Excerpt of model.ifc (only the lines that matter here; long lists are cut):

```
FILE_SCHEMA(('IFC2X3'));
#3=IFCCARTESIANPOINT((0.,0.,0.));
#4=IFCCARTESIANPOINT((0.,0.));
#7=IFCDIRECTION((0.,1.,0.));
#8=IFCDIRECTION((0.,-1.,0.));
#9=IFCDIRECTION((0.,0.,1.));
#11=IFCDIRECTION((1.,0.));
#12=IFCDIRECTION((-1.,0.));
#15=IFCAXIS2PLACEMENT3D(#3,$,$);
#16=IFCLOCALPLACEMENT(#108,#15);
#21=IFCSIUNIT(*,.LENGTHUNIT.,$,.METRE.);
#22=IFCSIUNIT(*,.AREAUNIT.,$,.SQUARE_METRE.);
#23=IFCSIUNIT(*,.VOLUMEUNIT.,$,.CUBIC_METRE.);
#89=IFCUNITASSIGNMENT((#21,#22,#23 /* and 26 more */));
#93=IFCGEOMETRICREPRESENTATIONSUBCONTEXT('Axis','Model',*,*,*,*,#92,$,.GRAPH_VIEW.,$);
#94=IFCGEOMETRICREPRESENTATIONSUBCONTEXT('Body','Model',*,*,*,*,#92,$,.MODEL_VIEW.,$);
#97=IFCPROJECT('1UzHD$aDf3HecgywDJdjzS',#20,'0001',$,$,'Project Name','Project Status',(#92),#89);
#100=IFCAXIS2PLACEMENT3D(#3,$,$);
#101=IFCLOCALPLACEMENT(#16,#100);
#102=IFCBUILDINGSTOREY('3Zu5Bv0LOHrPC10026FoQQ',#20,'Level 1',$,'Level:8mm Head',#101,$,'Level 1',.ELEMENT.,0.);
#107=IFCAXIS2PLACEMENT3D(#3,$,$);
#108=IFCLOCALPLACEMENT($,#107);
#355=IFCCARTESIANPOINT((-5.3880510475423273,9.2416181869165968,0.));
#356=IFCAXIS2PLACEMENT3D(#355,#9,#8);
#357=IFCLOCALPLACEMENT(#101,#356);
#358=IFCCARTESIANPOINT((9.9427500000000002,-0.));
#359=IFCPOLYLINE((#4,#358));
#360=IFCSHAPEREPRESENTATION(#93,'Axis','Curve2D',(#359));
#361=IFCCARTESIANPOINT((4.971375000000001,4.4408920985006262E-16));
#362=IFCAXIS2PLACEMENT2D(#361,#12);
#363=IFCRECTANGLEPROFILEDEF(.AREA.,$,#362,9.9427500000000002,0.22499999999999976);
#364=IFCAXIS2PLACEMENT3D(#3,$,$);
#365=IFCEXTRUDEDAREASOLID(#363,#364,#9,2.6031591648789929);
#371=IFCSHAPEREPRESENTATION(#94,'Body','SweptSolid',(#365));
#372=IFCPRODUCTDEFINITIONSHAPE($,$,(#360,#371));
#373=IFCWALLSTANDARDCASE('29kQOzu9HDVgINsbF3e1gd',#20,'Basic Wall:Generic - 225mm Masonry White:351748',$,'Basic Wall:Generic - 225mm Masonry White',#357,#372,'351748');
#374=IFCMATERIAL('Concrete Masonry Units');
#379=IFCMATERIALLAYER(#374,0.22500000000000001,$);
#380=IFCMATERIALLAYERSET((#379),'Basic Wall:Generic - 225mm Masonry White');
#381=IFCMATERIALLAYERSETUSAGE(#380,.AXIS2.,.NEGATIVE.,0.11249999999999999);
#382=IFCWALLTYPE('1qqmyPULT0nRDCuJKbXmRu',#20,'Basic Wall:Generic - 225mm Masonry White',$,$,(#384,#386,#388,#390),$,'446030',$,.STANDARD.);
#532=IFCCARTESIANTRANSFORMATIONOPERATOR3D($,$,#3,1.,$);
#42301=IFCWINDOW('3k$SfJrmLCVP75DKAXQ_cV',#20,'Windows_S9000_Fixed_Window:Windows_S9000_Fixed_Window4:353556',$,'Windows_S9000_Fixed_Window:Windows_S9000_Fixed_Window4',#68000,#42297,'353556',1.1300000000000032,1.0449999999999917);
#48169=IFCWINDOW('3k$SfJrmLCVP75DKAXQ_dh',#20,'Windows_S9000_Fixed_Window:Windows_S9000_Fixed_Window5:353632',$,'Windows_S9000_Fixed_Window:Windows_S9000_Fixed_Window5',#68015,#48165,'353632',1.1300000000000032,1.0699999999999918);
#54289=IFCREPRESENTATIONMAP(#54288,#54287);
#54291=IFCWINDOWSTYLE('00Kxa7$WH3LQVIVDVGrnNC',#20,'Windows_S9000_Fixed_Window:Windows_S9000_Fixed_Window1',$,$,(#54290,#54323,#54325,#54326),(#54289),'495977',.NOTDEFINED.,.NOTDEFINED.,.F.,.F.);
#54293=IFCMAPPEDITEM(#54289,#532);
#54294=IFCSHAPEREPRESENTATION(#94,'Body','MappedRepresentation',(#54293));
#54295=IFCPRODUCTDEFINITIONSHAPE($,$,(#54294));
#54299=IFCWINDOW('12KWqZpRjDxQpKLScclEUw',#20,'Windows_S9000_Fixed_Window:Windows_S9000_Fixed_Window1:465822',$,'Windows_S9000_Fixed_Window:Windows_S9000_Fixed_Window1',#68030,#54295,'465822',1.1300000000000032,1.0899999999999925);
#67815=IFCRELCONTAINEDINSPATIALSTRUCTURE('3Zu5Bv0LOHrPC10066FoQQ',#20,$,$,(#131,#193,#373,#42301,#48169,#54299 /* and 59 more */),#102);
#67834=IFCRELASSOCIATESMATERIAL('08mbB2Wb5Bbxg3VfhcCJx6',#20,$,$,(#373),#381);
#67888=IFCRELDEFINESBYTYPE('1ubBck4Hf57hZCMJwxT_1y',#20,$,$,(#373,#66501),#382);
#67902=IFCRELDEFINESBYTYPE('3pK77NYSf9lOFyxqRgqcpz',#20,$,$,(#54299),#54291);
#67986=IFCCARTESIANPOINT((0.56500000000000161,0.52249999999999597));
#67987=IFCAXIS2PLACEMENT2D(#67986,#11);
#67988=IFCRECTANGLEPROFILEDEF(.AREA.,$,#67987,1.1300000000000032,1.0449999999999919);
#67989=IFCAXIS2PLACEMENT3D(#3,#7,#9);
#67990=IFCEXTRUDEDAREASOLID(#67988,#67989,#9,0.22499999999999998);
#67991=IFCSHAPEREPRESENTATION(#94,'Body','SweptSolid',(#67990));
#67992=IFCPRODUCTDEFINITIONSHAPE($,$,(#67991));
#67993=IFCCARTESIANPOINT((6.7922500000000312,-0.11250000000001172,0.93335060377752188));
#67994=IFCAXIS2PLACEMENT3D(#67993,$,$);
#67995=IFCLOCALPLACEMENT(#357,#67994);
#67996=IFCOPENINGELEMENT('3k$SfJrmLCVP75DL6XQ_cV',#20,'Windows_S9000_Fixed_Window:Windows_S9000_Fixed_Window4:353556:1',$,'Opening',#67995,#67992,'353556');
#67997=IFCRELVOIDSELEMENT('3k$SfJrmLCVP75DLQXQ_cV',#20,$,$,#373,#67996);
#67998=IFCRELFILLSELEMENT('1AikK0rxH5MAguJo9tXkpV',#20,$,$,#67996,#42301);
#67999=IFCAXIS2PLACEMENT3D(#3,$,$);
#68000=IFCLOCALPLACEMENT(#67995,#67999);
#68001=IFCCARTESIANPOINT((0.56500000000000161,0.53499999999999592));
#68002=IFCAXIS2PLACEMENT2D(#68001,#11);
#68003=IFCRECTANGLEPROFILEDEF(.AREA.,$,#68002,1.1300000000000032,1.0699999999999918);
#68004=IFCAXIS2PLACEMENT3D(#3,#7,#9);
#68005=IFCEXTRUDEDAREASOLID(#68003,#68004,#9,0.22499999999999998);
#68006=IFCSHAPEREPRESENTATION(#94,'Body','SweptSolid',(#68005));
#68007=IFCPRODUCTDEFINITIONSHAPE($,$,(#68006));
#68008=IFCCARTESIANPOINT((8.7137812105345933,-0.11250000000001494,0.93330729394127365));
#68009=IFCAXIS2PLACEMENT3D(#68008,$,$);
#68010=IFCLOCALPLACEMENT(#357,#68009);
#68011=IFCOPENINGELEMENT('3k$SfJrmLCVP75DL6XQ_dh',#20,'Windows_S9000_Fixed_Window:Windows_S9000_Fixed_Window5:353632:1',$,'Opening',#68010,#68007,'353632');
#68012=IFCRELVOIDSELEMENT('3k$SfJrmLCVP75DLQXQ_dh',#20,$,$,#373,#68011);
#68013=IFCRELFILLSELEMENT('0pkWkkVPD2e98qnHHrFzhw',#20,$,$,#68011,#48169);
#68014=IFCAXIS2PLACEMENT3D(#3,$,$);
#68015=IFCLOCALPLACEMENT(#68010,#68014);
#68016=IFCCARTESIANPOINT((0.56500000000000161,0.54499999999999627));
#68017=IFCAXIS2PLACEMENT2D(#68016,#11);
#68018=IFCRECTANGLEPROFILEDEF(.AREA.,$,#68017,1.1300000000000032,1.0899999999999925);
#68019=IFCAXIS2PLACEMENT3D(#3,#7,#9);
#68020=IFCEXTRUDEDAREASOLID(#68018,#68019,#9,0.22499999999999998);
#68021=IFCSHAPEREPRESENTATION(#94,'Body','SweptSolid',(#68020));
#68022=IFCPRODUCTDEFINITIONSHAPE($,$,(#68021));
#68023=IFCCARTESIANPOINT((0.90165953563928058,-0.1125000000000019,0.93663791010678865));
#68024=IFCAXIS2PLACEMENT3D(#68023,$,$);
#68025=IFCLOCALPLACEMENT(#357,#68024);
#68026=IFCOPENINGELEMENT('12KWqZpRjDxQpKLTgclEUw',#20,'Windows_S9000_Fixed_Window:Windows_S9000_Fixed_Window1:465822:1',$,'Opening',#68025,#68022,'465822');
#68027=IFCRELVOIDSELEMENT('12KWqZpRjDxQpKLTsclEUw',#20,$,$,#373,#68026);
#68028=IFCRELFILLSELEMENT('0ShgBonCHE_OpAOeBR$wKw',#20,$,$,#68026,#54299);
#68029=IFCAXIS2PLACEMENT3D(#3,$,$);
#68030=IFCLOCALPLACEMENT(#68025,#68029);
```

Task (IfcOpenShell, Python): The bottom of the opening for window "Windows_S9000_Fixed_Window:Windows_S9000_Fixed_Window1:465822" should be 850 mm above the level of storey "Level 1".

```python
import numpy as np
import ifcopenshell
import ifcopenshell.api.geometry
import ifcopenshell.geom
import ifcopenshell.util.element
import ifcopenshell.util.placement
import ifcopenshell.util.shape
import ifcopenshell.util.unit

model = ifcopenshell.open("model.ifc")
unit_scale = ifcopenshell.util.unit.calculate_unit_scale(model)

window = model.by_guid("12KWqZpRjDxQpKLScclEUw")
opening = window.FillsVoids[0].RelatingOpeningElement
storey = ifcopenshell.util.element.get_container(window, ifc_class="IfcBuildingStorey")
level = ifcopenshell.util.placement.get_local_placement(storey.ObjectPlacement)[2, 3]

# The opening's origin need not be at the sill, so measure its lowest point.
shape = ifcopenshell.geom.create_shape(ifcopenshell.geom.settings(), opening)
bottom = ifcopenshell.util.shape.get_shape_bottom_elevation(shape, shape.geometry) / unit_scale
dz = level + 0.85 / unit_scale - bottom

shift = np.array([0.0, 0.0, dz])
# The window is placed relative to its opening, so it follows when the opening moves.
matrix = ifcopenshell.util.placement.get_local_placement(opening.ObjectPlacement)
matrix[:3, 3] += shift
ifcopenshell.api.geometry.edit_object_placement(
    model, product=opening, matrix=matrix, is_si=False, should_transform_children=True
)

print(f"moved by {dz * unit_scale:+.3f} m")

model.write("model_rev.ifc")
```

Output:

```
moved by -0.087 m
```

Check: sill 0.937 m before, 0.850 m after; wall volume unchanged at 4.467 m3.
